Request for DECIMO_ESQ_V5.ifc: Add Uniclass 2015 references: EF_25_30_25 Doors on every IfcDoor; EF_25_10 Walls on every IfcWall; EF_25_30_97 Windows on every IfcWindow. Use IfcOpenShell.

First a look at what the model holds.

```python
import ifcopenshell

model = ifcopenshell.open("DECIMO_ESQ_V5.ifc")
print(model.schema)
print("classifications:", [c.Name for c in model.by_type("IfcClassification")])
for ifc_class in ("IfcDoor", "IfcRoof", "IfcStair", "IfcWall", "IfcWindow"):
    print(ifc_class, len(model.by_type(ifc_class)))
```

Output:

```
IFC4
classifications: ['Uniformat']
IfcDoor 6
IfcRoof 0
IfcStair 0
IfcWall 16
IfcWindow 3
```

```python
import ifcopenshell
import ifcopenshell.api.classification

model = ifcopenshell.open("DECIMO_ESQ_V5.ifc")

system = ifcopenshell.api.classification.add_classification(model, classification="Uniclass 2015")

codes = {
    "IfcDoor": ("EF_25_30_25", "Doors"),
    "IfcWall": ("EF_25_10", "Walls"),
    "IfcWindow": ("EF_25_30_97", "Windows"),
}
for ifc_class, (code, name) in codes.items():
    products = model.by_type(ifc_class)
    ifcopenshell.api.classification.add_reference(
        model, products=products, classification=system, identification=code, name=name
    )
    print(code, len(products))

model.write("DECIMO_ESQ_V5_rev.ifc")
```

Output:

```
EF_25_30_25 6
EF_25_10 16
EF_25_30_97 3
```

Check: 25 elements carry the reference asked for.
